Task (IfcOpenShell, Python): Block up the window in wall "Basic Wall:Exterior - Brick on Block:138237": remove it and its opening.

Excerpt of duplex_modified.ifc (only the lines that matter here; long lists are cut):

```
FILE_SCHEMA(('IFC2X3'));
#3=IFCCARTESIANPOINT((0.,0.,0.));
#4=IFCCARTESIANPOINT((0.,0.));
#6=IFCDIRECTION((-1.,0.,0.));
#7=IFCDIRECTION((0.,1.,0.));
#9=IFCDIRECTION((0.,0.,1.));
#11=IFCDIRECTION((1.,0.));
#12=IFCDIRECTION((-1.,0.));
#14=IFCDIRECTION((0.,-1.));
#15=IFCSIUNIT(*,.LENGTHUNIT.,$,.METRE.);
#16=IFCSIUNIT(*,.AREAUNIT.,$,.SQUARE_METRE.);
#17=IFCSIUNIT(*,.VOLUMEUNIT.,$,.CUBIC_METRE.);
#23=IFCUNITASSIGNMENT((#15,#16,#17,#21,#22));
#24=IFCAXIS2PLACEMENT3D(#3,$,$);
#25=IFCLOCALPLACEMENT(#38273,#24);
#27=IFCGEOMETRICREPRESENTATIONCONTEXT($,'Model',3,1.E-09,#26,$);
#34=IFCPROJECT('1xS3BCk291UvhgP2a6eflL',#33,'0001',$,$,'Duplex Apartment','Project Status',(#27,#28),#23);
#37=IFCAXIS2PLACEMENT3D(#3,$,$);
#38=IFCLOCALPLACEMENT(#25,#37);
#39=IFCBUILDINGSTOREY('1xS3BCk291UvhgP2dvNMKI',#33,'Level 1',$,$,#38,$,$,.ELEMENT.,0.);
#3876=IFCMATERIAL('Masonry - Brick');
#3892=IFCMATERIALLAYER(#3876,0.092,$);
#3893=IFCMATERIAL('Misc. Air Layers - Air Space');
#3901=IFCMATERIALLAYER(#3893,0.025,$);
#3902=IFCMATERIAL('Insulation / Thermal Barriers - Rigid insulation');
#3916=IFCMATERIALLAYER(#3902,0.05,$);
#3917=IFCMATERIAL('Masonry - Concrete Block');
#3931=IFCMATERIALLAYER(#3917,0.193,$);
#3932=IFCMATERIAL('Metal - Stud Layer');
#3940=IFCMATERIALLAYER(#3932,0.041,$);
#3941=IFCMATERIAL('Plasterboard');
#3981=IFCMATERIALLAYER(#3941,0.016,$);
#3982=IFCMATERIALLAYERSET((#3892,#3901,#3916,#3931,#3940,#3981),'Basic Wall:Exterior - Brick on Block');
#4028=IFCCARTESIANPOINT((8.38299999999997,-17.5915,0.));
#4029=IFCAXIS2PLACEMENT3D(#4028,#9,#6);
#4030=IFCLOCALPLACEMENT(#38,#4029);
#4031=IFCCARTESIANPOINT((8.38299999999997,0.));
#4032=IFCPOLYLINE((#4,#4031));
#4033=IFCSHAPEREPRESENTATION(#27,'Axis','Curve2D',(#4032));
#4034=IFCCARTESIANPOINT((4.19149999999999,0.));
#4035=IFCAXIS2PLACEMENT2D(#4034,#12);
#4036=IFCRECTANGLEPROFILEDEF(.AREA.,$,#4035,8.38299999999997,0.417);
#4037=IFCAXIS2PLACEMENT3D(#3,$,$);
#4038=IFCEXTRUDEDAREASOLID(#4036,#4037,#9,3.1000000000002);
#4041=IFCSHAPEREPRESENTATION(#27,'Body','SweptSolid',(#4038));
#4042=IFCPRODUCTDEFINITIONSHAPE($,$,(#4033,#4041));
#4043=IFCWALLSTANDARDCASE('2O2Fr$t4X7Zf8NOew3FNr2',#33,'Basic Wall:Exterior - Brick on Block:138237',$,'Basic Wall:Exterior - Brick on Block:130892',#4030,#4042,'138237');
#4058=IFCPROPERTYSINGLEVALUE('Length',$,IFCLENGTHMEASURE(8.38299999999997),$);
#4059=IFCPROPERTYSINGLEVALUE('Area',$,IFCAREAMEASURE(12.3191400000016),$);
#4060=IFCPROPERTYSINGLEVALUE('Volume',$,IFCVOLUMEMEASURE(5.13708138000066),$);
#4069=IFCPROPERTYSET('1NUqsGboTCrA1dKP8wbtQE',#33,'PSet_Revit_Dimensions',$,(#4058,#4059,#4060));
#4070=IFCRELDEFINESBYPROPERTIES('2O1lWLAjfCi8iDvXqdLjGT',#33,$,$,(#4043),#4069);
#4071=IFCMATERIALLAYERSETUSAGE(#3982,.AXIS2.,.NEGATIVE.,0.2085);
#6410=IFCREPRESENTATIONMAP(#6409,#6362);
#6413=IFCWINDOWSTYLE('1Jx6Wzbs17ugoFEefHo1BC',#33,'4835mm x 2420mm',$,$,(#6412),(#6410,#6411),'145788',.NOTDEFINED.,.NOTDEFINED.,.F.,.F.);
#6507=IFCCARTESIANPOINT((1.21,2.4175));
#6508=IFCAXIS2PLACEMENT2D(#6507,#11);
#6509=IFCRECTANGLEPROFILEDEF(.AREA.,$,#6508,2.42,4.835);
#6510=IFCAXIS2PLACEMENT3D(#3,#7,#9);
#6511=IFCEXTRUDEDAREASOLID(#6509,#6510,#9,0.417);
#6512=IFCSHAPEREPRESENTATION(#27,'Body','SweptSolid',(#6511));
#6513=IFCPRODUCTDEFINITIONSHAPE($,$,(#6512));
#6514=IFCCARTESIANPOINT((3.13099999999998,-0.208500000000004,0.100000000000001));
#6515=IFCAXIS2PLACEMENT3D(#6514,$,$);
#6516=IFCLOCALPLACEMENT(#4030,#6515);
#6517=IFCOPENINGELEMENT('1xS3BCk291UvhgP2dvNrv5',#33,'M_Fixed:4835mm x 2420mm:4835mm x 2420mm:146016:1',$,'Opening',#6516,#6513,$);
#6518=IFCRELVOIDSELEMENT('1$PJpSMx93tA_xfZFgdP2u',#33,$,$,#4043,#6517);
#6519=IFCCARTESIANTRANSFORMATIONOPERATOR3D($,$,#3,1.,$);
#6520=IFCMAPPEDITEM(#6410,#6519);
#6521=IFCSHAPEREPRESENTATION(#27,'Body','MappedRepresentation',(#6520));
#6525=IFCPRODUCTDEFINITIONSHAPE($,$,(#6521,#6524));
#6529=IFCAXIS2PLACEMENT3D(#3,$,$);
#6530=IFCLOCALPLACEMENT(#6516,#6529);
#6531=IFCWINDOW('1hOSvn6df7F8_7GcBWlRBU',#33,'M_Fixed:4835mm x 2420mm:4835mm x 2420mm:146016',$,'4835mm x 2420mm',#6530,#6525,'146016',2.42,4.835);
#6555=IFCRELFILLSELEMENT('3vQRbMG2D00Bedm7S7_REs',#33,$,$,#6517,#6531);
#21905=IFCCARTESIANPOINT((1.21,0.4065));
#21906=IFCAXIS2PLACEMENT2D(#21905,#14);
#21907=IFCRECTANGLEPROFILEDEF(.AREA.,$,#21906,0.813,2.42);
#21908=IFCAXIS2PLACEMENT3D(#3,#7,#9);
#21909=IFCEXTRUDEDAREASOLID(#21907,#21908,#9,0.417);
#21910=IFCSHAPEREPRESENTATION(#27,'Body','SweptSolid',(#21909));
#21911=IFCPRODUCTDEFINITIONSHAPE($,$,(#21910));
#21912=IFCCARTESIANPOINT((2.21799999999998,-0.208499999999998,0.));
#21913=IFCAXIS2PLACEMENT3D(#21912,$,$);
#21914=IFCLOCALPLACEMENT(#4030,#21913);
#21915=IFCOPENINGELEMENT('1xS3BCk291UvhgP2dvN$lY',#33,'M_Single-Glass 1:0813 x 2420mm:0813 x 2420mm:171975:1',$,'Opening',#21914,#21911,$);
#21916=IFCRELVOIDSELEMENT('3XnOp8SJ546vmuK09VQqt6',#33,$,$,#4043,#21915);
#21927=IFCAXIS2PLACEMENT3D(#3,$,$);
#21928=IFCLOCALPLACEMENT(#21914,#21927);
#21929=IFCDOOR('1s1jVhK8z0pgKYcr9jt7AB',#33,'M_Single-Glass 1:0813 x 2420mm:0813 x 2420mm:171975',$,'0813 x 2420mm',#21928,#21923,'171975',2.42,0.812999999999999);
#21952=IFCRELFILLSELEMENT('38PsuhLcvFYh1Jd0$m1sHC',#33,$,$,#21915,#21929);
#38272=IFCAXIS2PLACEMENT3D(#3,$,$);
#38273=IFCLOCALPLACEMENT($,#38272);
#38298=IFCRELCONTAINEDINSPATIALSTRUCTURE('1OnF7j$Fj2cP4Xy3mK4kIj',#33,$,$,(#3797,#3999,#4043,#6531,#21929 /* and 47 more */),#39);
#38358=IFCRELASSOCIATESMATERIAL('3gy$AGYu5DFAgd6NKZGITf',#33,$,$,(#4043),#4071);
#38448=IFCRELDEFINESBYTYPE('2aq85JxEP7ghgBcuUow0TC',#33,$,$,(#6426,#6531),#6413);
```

```python
import ifcopenshell
import ifcopenshell.api.feature
import ifcopenshell.api.pset
import ifcopenshell.api.root
import ifcopenshell.geom
import ifcopenshell.util.element
import ifcopenshell.util.shape
import ifcopenshell.util.unit

model = ifcopenshell.open("duplex_modified.ifc")
area_scale = ifcopenshell.util.unit.calculate_unit_scale(model, "AREAUNIT")
volume_scale = ifcopenshell.util.unit.calculate_unit_scale(model, "VOLUMEUNIT")
settings = ifcopenshell.geom.settings()


def volume(element):
    """Net volume in cubic metres, openings subtracted."""
    shape = ifcopenshell.geom.create_shape(settings, element)
    return ifcopenshell.util.shape.get_volume(shape.geometry)


window = model.by_guid("1hOSvn6df7F8_7GcBWlRBU")
opening = window.FillsVoids[0].RelatingOpeningElement
wall = opening.VoidsElements[0].RelatingBuildingElement
before = volume(wall)

ifcopenshell.api.root.remove_product(model, product=window)
ifcopenshell.api.feature.remove_feature(model, feature=opening)

after = volume(wall)
thickness = 0.417  # wall thickness in metres

# Update the wall's stored quantities.
pset = model.by_id(ifcopenshell.util.element.get_pset(wall, "PSet_Revit_Dimensions", should_inherit=False)["id"])
ifcopenshell.api.pset.edit_pset(model, pset=pset, properties={
    "Area": model.create_entity("IfcAreaMeasure", after / thickness / area_scale),
    "Volume": model.create_entity("IfcVolumeMeasure", after / volume_scale),
})

print(f"wall volume {before:.3f} -> {after:.3f} m3")

model.write("duplex_modified_rev.ifc")
```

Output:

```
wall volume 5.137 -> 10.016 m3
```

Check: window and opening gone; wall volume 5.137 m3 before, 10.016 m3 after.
